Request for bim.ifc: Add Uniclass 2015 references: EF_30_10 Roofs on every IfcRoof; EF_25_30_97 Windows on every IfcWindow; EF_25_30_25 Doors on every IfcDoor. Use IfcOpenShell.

First a look at what the model holds.

```python
import ifcopenshell

model = ifcopenshell.open("bim.ifc")
print(model.schema)
print("classifications:", [c.Name for c in model.by_type("IfcClassification")])
for ifc_class in ("IfcDoor", "IfcRoof", "IfcStair", "IfcWall", "IfcWindow"):
    print(ifc_class, len(model.by_type(ifc_class)))
```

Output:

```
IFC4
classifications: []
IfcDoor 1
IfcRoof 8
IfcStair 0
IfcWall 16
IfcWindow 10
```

```python
import ifcopenshell
import ifcopenshell.api.classification

model = ifcopenshell.open("bim.ifc")

system = ifcopenshell.api.classification.add_classification(model, classification="Uniclass 2015")

codes = {
    "IfcRoof": ("EF_30_10", "Roofs"),
    "IfcWindow": ("EF_25_30_97", "Windows"),
    "IfcDoor": ("EF_25_30_25", "Doors"),
}
for ifc_class, (code, name) in codes.items():
    products = model.by_type(ifc_class)
    ifcopenshell.api.classification.add_reference(
        model, products=products, classification=system, identification=code, name=name
    )
    print(code, len(products))

model.write("bim-out.ifc")
```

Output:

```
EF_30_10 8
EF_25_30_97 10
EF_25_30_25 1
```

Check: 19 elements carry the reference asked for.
